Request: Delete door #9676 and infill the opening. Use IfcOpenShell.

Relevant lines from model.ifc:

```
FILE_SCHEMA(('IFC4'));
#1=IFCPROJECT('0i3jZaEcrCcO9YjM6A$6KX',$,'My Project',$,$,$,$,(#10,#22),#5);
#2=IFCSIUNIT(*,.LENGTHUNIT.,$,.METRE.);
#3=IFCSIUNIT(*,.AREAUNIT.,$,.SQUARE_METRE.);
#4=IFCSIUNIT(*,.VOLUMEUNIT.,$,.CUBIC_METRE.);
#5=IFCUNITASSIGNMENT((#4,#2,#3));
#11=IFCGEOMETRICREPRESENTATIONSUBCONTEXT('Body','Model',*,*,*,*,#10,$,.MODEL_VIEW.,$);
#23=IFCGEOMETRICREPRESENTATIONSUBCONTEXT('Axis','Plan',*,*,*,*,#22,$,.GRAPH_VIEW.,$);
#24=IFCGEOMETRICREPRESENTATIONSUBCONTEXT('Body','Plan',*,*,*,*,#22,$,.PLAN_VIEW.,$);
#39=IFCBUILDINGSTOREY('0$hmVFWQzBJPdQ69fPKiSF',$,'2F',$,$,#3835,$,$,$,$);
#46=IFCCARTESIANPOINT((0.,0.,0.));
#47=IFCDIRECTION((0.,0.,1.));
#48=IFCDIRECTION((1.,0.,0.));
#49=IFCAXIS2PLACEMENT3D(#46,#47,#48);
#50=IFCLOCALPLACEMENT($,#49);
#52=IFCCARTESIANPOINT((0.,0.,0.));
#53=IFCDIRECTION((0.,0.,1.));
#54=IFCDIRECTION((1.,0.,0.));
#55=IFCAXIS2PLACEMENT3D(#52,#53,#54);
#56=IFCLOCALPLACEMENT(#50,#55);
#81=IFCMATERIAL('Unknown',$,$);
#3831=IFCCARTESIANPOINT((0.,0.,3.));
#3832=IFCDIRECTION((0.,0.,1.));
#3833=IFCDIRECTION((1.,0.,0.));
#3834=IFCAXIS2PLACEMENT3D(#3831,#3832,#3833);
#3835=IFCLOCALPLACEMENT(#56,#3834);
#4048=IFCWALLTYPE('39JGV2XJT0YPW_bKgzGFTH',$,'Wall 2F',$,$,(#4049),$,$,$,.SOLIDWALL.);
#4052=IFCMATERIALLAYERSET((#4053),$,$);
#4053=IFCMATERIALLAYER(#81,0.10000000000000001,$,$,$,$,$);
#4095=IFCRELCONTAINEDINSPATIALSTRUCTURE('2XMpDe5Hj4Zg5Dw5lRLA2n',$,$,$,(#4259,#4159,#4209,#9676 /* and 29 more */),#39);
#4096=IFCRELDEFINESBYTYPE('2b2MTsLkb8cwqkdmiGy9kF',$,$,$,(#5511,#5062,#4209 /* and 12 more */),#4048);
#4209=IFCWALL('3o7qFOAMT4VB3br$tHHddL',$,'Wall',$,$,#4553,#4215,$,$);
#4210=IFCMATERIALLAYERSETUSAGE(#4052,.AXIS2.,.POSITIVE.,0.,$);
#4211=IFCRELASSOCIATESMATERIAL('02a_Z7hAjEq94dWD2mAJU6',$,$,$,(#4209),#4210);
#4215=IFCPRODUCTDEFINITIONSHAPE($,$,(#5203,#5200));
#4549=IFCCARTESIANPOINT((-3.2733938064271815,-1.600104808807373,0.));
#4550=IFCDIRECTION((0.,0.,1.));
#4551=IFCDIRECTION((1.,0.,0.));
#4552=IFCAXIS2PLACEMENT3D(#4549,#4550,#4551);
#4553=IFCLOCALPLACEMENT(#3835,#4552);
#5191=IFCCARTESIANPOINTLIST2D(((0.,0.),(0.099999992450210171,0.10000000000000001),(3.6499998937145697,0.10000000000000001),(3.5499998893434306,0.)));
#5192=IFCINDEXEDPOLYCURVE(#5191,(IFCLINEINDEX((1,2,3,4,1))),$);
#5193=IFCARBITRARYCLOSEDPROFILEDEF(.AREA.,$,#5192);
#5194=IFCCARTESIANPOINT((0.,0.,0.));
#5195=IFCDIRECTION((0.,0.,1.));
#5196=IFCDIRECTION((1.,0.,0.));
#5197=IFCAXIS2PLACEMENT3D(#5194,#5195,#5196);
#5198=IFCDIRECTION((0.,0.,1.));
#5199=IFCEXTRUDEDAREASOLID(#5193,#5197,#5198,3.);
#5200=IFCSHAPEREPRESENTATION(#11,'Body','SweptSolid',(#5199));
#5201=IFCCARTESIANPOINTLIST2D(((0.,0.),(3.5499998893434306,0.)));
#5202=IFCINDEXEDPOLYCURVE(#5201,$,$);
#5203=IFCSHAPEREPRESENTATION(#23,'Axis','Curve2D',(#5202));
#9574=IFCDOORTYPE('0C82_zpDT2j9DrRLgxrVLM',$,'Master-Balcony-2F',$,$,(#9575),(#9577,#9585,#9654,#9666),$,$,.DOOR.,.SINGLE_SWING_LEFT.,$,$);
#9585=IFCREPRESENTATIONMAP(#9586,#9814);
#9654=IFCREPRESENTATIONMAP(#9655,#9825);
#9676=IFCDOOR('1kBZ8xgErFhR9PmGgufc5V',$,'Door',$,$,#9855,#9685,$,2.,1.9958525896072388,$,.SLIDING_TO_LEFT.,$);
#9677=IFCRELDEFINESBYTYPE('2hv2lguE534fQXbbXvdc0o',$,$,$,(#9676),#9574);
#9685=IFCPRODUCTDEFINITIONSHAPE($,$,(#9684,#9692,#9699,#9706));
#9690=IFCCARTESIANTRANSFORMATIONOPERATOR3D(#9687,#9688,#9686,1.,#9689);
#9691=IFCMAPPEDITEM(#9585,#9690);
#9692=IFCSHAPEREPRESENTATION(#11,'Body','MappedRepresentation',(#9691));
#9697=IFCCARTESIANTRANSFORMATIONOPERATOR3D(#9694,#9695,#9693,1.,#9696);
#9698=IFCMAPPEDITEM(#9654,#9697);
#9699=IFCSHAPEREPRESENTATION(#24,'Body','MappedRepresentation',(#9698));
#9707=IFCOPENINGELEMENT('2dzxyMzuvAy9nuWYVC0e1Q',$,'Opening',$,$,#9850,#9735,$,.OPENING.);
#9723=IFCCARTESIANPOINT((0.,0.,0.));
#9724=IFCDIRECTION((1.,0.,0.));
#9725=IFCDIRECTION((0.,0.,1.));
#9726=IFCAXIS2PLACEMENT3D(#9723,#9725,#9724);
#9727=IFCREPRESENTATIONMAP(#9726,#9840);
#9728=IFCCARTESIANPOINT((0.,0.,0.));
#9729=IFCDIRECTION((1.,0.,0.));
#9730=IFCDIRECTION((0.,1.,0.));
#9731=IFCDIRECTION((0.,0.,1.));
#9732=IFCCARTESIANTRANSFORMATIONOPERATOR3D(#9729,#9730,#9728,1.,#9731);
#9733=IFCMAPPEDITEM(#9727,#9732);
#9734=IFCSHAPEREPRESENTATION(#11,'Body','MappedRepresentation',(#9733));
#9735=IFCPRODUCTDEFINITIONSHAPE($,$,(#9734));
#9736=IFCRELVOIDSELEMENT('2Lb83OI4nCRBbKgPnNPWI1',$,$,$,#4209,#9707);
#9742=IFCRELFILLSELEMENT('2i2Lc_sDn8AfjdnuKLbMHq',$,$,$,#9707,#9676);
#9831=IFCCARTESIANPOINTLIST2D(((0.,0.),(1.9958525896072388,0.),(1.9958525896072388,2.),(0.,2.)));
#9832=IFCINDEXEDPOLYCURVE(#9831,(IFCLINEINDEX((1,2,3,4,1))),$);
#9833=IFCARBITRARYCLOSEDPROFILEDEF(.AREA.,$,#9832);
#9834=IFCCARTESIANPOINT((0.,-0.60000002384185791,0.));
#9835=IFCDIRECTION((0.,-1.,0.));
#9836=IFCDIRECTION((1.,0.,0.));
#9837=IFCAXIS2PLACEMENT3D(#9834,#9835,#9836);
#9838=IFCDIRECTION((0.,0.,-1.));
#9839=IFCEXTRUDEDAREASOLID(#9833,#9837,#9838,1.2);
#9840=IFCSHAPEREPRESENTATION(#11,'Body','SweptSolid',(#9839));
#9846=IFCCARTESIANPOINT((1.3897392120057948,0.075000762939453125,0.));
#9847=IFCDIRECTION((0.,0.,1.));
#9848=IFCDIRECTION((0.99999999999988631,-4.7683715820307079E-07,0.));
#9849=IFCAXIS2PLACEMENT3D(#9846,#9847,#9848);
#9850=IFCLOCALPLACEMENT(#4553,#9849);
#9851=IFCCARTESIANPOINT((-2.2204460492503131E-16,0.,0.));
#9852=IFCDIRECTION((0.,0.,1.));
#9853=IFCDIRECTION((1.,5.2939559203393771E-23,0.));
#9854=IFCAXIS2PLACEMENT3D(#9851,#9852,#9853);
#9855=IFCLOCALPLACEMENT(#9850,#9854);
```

```python
import ifcopenshell
import ifcopenshell.api.feature
import ifcopenshell.api.root
import ifcopenshell.geom
import ifcopenshell.util.shape

model = ifcopenshell.open("model.ifc")
settings = ifcopenshell.geom.settings()


def volume(element):
    """Net volume in cubic metres, openings subtracted."""
    shape = ifcopenshell.geom.create_shape(settings, element)
    return ifcopenshell.util.shape.get_volume(shape.geometry)


door = model.by_id(9676)
opening = door.FillsVoids[0].RelatingOpeningElement
wall = opening.VoidsElements[0].RelatingBuildingElement
before = volume(wall)

ifcopenshell.api.root.remove_product(model, product=door)
ifcopenshell.api.feature.remove_feature(model, feature=opening)

after = volume(wall)

print(f"wall volume {before:.3f} -> {after:.3f} m3")

model.write("model_updated.ifc")
```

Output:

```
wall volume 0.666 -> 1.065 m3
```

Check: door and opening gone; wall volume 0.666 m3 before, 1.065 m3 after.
